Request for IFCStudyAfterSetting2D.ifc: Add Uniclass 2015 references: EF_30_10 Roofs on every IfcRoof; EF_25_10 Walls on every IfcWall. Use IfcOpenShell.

First a look at what the model holds.

```python
import ifcopenshell

model = ifcopenshell.open("IFCStudyAfterSetting2D.ifc")
print(model.schema)
print("classifications:", [c.Name for c in model.by_type("IfcClassification")])
for ifc_class in ("IfcDoor", "IfcRoof", "IfcStair", "IfcWall", "IfcWindow"):
    print(ifc_class, len(model.by_type(ifc_class)))
```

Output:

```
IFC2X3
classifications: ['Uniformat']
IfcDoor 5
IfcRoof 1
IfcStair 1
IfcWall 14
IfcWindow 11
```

```python
import ifcopenshell
import ifcopenshell.api.classification

model = ifcopenshell.open("IFCStudyAfterSetting2D.ifc")

# IFC2X3 requires Source and Edition and has no link from the project to the system.
system = model.create_entity("IfcClassification", Source="NBS", Edition="2015", Name="Uniclass 2015")

codes = {
    "IfcRoof": ("EF_30_10", "Roofs"),
    "IfcWall": ("EF_25_10", "Walls"),
}
for ifc_class, (code, name) in codes.items():
    products = model.by_type(ifc_class)
    ifcopenshell.api.classification.add_reference(
        model, products=products, classification=system, identification=code, name=name
    )
    print(code, len(products))

model.write("IFCStudyAfterSetting2D-out.ifc")
```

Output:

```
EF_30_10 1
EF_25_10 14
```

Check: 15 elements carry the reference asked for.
